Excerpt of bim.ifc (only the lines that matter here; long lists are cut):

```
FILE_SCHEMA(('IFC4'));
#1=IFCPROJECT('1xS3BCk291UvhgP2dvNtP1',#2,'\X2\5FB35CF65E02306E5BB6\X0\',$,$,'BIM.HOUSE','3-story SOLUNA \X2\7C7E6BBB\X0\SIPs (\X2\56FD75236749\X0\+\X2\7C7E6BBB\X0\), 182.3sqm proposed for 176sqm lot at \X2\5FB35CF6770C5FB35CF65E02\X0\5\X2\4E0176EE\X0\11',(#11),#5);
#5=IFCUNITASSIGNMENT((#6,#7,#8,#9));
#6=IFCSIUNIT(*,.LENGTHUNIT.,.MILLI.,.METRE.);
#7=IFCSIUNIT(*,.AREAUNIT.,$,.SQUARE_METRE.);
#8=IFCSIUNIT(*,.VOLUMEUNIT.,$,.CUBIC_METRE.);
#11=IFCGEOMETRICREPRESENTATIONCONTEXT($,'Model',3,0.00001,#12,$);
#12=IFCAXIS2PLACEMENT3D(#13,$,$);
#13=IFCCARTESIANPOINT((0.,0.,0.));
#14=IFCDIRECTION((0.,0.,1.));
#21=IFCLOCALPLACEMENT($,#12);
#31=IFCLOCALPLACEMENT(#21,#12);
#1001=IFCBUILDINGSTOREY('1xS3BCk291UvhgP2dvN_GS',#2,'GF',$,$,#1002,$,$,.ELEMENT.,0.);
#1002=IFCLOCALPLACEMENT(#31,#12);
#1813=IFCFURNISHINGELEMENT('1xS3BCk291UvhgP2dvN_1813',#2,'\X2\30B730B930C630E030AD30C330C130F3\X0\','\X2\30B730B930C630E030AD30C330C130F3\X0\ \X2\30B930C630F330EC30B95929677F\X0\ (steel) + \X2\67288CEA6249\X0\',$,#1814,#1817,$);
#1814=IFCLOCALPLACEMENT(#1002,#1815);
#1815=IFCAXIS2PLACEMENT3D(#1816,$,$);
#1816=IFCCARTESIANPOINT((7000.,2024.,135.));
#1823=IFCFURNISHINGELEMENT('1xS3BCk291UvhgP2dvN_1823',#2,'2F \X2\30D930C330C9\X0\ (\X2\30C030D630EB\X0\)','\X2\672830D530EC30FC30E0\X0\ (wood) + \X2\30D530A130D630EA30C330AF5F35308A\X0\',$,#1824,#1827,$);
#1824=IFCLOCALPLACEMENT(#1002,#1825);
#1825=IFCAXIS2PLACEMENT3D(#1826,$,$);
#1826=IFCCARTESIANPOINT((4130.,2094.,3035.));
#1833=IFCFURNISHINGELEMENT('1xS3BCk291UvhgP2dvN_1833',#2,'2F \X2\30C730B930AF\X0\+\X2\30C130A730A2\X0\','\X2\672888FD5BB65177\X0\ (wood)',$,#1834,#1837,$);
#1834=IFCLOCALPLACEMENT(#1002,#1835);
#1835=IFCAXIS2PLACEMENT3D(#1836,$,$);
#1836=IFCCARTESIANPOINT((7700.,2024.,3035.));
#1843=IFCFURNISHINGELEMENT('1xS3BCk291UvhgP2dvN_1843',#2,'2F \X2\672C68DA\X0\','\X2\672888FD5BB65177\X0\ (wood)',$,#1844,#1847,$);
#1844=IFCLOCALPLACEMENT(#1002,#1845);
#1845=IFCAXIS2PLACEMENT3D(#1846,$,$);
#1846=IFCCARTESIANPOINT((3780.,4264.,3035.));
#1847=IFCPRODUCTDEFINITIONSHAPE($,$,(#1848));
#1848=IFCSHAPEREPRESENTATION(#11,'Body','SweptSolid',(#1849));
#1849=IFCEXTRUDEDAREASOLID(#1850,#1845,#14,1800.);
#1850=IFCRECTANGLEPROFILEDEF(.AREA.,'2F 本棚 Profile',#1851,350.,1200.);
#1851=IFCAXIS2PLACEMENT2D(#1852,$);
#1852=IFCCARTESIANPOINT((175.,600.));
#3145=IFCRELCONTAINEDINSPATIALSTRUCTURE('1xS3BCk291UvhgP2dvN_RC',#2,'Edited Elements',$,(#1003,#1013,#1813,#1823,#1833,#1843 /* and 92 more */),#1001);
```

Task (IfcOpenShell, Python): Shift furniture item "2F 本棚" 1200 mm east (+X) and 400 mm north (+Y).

```python
import ifcopenshell
import ifcopenshell.api.geometry
import ifcopenshell.util.placement
import ifcopenshell.util.unit

model = ifcopenshell.open("bim.ifc")
unit_scale = ifcopenshell.util.unit.calculate_unit_scale(model)

item = model.by_guid("1xS3BCk291UvhgP2dvN_1843")
matrix = ifcopenshell.util.placement.get_local_placement(item.ObjectPlacement)
matrix[0, 3] += 1.2 / unit_scale
matrix[1, 3] += 0.4 / unit_scale
ifcopenshell.api.geometry.edit_object_placement(model, product=item, matrix=matrix, is_si=False)

print(ifcopenshell.util.placement.get_local_placement(item.ObjectPlacement).round(3) + 0.0)

model.write("bim_rev.ifc")
```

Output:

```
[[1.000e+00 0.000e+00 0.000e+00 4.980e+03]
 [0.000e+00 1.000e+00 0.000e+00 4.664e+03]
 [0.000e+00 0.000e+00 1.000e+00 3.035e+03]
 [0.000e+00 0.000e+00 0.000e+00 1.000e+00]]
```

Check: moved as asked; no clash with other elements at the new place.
